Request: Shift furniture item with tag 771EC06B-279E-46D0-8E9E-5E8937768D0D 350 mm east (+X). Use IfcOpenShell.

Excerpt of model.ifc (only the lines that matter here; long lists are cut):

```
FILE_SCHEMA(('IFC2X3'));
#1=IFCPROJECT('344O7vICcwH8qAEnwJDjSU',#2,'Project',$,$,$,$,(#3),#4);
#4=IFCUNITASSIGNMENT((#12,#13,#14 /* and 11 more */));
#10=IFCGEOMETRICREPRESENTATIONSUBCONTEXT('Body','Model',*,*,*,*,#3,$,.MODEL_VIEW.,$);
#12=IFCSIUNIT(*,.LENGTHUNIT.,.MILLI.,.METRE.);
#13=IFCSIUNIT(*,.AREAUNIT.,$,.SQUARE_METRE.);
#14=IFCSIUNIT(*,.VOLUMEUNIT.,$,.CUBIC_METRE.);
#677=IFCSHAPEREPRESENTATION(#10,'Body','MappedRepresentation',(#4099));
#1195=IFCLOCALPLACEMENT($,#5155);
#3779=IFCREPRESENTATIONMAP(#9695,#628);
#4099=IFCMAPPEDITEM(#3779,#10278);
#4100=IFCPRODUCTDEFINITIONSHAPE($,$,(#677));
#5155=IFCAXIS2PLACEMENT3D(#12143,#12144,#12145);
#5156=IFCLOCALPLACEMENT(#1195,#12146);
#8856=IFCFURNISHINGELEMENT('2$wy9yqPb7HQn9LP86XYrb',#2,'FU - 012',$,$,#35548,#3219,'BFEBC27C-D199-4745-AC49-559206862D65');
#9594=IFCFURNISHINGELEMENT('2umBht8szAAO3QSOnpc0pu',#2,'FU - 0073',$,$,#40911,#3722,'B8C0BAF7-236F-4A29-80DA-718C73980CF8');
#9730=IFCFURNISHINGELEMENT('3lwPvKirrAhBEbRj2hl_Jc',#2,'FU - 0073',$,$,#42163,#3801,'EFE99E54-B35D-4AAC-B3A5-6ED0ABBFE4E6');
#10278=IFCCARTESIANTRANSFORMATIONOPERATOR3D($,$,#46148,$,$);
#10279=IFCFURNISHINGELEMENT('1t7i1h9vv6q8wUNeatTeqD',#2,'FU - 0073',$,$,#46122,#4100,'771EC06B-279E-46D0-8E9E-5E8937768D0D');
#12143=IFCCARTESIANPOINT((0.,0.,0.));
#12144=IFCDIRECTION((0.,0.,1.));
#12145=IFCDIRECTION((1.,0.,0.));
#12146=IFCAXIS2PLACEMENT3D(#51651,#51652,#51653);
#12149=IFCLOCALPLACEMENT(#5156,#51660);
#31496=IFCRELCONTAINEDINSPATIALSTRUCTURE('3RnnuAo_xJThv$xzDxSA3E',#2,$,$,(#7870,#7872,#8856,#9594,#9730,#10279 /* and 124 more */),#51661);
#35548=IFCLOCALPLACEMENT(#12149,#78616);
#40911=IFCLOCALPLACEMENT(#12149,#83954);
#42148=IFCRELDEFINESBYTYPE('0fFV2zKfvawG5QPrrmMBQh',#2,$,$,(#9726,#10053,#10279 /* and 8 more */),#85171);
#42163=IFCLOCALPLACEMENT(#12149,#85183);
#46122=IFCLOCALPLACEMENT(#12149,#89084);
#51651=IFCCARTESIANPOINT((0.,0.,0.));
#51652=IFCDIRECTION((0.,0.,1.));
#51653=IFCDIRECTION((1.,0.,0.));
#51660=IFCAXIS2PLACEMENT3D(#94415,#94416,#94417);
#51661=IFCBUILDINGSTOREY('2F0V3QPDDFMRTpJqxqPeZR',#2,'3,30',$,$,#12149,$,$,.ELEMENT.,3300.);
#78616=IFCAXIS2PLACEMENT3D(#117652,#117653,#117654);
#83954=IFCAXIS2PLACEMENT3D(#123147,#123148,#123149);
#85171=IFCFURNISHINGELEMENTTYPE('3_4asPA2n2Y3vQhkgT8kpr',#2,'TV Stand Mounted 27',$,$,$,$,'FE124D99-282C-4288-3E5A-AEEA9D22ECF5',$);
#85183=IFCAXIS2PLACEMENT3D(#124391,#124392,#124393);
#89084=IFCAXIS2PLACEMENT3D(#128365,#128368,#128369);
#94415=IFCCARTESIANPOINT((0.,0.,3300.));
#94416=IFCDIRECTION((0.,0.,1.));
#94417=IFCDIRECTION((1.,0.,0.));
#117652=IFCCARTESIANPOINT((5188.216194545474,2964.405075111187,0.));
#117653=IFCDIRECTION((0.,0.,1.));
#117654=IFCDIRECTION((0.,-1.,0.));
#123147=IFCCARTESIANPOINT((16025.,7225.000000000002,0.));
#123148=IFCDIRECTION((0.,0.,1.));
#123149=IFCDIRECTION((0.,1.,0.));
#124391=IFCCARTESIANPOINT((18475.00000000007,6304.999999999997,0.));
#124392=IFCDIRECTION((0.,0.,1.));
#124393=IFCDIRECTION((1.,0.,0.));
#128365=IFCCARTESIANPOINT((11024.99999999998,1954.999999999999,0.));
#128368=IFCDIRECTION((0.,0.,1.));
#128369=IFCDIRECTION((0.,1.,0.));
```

```python
import ifcopenshell
import ifcopenshell.api.geometry
import ifcopenshell.util.placement

model = ifcopenshell.open("model.ifc")

item = model.by_guid("1t7i1h9vv6q8wUNeatTeqD")
matrix = ifcopenshell.util.placement.get_local_placement(item.ObjectPlacement)
matrix[0, 3] += 350.0
ifcopenshell.api.geometry.edit_object_placement(model, product=item, matrix=matrix, is_si=False)

print(ifcopenshell.util.placement.get_local_placement(item.ObjectPlacement).round(3) + 0.0)

model.write("model_edited.ifc")
```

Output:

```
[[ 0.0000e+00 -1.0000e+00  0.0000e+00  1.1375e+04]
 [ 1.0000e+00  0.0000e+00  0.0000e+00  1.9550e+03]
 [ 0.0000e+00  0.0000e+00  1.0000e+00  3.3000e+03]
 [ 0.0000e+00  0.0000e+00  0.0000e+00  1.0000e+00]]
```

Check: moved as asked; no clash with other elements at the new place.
